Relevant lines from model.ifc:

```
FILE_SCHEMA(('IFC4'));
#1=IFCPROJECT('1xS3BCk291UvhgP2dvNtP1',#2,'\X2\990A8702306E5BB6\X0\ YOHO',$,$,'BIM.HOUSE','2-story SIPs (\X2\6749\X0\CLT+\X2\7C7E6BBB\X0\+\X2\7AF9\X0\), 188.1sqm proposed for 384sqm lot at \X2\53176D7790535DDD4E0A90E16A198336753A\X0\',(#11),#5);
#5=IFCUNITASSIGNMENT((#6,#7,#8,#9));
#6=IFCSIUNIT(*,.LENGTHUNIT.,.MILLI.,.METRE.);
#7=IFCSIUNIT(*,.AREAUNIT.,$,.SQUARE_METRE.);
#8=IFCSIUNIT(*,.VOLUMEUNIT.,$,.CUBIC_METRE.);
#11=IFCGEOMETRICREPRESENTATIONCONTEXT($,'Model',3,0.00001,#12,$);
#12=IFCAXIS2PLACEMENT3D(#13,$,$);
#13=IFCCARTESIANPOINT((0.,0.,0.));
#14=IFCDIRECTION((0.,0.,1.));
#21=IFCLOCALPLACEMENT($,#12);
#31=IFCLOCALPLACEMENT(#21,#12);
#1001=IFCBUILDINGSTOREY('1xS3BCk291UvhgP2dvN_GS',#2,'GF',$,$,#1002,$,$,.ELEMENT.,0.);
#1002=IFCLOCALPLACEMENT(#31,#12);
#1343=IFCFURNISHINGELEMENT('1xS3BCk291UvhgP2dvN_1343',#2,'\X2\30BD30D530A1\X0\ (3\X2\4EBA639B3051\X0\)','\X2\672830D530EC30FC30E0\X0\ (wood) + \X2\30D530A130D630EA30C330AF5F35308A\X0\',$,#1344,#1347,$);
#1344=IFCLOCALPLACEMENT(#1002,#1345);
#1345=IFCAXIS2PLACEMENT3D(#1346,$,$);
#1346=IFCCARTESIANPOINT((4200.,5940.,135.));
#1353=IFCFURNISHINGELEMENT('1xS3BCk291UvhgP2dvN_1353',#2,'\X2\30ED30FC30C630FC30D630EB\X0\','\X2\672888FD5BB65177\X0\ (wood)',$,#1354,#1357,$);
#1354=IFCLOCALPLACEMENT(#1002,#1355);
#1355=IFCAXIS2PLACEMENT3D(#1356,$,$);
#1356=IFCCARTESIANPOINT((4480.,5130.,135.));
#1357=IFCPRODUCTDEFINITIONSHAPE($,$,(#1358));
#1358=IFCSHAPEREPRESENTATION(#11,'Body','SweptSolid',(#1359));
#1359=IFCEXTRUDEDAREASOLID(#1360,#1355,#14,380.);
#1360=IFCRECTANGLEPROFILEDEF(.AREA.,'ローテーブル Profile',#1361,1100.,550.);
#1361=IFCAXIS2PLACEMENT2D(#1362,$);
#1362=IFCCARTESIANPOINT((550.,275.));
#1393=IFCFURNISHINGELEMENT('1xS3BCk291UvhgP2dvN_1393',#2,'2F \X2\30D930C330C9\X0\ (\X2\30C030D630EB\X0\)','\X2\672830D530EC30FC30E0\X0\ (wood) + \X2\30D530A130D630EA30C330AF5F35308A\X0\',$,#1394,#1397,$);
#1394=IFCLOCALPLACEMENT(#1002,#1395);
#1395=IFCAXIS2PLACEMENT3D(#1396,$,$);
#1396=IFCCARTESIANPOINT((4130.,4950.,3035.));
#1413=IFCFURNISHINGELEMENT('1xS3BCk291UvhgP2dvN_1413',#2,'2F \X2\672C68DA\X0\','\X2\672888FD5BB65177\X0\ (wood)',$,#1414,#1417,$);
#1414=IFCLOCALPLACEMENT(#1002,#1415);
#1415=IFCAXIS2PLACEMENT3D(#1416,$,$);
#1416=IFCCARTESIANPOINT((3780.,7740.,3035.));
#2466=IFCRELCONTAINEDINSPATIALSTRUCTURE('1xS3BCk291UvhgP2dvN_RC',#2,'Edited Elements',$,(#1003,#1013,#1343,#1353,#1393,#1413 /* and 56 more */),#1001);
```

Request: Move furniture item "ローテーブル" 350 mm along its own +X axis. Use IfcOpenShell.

```python
import ifcopenshell
import ifcopenshell.api.geometry
import ifcopenshell.util.placement
import ifcopenshell.util.unit

model = ifcopenshell.open("model.ifc")
unit_scale = ifcopenshell.util.unit.calculate_unit_scale(model)

item = model.by_id(1353)
matrix = ifcopenshell.util.placement.get_local_placement(item.ObjectPlacement)
matrix[:3, 3] += matrix[:3, 0] * 0.35 / unit_scale
ifcopenshell.api.geometry.edit_object_placement(model, product=item, matrix=matrix, is_si=False)

print(ifcopenshell.util.placement.get_local_placement(item.ObjectPlacement).round(3) + 0.0)

model.write("model-out.ifc")
```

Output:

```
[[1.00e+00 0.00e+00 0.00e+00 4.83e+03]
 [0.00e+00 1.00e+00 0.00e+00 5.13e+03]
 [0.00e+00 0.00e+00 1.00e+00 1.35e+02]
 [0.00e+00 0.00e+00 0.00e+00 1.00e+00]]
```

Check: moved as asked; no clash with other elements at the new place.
